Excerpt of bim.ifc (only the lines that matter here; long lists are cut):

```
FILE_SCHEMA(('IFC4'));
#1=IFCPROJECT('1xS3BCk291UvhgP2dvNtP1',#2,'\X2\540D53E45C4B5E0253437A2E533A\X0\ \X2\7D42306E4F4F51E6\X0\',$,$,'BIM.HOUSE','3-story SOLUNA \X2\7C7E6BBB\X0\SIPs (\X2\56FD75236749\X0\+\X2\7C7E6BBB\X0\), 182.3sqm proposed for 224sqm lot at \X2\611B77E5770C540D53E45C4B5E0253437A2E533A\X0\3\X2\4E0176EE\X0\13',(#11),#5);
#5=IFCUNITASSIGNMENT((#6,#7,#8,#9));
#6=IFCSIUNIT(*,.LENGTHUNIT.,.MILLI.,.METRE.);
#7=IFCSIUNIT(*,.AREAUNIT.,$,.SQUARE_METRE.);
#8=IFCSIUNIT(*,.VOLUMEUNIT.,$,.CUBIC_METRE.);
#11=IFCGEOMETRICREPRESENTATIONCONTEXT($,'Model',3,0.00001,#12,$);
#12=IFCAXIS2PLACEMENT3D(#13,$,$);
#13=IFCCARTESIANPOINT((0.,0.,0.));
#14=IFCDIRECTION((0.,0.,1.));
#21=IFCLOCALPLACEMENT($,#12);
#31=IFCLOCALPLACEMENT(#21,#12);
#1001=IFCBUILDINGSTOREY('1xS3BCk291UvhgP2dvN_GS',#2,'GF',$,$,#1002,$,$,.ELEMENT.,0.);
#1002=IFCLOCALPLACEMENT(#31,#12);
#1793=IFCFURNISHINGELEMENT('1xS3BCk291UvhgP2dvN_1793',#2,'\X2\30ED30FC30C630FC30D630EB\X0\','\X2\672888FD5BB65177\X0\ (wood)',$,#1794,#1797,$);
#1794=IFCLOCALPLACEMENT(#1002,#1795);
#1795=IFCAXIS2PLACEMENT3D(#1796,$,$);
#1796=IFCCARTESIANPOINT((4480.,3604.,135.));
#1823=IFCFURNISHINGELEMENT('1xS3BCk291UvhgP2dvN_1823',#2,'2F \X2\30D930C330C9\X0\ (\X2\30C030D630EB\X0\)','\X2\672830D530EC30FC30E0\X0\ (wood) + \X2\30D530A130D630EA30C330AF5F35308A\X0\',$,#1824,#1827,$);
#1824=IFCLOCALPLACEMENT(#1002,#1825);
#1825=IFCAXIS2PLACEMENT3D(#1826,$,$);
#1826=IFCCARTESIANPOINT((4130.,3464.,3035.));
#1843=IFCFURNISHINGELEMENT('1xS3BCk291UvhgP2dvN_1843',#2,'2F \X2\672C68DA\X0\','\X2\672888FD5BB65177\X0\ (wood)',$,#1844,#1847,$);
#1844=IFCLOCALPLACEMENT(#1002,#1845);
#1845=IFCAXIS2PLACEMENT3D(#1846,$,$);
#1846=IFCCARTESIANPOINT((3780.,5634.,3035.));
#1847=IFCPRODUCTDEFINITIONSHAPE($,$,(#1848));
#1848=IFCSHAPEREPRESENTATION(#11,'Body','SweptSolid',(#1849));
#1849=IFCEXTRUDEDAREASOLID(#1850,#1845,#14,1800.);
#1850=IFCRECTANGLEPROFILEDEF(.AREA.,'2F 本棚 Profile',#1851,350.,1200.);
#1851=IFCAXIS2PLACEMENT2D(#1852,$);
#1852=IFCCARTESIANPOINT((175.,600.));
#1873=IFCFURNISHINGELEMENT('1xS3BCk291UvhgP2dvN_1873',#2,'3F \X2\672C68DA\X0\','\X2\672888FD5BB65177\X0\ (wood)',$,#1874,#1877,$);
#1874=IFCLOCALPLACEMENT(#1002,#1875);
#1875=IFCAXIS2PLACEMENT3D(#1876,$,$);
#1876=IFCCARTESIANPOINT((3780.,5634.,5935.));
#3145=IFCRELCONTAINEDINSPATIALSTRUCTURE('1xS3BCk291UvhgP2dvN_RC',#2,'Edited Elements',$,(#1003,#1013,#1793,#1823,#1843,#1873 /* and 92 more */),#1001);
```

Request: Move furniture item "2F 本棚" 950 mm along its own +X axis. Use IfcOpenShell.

```python
import ifcopenshell
import ifcopenshell.api.geometry
import ifcopenshell.util.placement

model = ifcopenshell.open("bim.ifc")

item = model.by_id(1843)
matrix = ifcopenshell.util.placement.get_local_placement(item.ObjectPlacement)
matrix[:3, 3] += matrix[:3, 0] * 950.0
ifcopenshell.api.geometry.edit_object_placement(model, product=item, matrix=matrix, is_si=False)

print(ifcopenshell.util.placement.get_local_placement(item.ObjectPlacement).round(3) + 0.0)

model.write("bim_rev.ifc")
```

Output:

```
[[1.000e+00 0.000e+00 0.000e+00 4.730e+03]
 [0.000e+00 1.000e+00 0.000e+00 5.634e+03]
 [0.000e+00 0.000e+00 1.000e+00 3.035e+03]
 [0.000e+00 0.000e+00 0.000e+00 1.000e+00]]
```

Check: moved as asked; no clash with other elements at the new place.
